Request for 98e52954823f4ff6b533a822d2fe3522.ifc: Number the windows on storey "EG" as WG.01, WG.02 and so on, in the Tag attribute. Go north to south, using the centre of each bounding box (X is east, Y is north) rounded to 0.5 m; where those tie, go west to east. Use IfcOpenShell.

First a look at what the model holds.

```python
import ifcopenshell
import ifcopenshell.util.element
import ifcopenshell.util.placement

model = ifcopenshell.open("98e52954823f4ff6b533a822d2fe3522.ifc")
print(model.schema)
storey = next(s for s in model.by_type("IfcBuildingStorey") if s.Name == "EG")
windows = [e for e in ifcopenshell.util.element.get_decomposition(storey) if e.is_a("IfcWindow")]
for e in sorted(windows, key=lambda e: e.id()):
    origin = ifcopenshell.util.placement.get_local_placement(e.ObjectPlacement)[:3, 3]
    print(e.id(), e.Tag, e.Name, origin.round(2) + 0.0, sep=" | ")
```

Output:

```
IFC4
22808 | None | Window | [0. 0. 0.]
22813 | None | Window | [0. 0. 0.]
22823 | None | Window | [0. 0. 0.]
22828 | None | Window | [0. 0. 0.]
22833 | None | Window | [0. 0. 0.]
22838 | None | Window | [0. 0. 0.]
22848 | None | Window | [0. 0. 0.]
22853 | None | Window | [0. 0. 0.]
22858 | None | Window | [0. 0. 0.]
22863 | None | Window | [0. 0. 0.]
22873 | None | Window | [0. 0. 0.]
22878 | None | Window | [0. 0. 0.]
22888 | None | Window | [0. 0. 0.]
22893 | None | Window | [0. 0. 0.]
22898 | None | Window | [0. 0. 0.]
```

```python
import ifcopenshell
import ifcopenshell.geom
import ifcopenshell.util.element
import ifcopenshell.util.shape

model = ifcopenshell.open("98e52954823f4ff6b533a822d2fe3522.ifc")
settings = ifcopenshell.geom.settings()
settings.set("use-world-coords", True)


def centre(element):
    shape = ifcopenshell.geom.create_shape(settings, element)
    return ifcopenshell.util.shape.get_bbox_centroid(shape.geometry)


storey = next(s for s in model.by_type("IfcBuildingStorey") if s.Name == "EG")
windows = [e for e in ifcopenshell.util.element.get_decomposition(storey) if e.is_a("IfcWindow")]

# Insertion points can sit at a corner or the storey origin, so sort by the geometry (in metres).
centres = {e: centre(e) for e in windows}
windows.sort(key=lambda e: (-round(centres[e][1] / 0.5), centres[e][0]))

for i, e in enumerate(windows, start=1):
    number = f"WG.{i:02d}"
    e.Tag = number
    print(e.id(), number)

model.write("98e52954823f4ff6b533a822d2fe3522_updated.ifc")
```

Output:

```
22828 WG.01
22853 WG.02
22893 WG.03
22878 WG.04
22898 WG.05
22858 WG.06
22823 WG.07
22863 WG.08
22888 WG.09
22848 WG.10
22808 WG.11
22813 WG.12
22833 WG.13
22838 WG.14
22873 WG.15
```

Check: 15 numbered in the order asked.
